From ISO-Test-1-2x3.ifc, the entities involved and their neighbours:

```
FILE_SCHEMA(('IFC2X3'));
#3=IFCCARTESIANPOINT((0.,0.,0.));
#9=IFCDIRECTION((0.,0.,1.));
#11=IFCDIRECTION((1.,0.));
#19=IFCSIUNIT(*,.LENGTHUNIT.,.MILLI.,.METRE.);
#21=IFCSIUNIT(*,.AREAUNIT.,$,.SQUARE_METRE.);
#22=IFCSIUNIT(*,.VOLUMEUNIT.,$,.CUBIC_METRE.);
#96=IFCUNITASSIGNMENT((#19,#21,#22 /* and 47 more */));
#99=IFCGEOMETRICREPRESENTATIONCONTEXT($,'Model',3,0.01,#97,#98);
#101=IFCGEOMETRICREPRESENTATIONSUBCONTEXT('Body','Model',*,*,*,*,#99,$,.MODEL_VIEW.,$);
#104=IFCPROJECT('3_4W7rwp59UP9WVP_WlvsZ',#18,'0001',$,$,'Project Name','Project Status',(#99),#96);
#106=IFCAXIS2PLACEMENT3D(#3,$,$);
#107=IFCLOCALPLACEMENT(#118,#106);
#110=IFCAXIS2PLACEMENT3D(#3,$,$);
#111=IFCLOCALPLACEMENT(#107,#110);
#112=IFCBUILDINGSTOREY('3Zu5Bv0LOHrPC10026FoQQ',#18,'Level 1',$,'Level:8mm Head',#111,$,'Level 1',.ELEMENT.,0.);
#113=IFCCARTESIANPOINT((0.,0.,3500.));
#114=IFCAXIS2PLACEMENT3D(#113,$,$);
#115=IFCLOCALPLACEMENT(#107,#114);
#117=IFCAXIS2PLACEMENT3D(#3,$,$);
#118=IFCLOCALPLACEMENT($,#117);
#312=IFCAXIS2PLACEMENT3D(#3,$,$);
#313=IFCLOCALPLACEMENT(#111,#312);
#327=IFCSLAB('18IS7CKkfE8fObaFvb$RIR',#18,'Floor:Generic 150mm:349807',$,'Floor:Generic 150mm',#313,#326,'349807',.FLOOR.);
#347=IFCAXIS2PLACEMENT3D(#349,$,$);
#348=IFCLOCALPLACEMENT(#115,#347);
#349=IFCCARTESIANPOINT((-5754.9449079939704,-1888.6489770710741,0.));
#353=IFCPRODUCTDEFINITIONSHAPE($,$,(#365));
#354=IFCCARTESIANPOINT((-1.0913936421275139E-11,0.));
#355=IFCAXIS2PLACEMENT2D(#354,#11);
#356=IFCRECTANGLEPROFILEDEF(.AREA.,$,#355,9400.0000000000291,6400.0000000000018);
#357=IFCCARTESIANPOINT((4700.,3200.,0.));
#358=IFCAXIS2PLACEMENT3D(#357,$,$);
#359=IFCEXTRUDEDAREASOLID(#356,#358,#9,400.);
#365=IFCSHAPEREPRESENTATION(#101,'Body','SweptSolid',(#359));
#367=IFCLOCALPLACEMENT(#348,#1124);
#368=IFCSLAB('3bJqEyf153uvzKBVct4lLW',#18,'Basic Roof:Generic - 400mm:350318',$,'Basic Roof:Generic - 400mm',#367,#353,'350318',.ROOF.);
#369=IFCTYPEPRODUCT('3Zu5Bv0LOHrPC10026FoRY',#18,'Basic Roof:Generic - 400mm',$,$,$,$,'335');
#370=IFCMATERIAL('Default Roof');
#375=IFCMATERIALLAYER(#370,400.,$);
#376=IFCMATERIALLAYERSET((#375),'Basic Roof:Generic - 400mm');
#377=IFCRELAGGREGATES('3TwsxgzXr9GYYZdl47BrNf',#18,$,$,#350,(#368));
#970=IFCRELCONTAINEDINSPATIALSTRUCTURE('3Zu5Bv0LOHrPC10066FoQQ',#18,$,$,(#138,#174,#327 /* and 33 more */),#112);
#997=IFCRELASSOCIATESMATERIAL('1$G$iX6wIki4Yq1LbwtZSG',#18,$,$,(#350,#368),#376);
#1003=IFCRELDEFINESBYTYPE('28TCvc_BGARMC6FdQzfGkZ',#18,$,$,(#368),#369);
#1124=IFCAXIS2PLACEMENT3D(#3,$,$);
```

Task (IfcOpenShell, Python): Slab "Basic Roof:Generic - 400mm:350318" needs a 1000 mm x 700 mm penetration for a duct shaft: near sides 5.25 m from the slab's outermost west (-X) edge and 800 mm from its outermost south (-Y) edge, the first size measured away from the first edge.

```python
import numpy as np
import ifcopenshell
import ifcopenshell.api.feature
import ifcopenshell.api.geometry
import ifcopenshell.api.root
import ifcopenshell.geom
import ifcopenshell.util.placement
import ifcopenshell.util.representation
import ifcopenshell.util.shape
import ifcopenshell.util.unit

model = ifcopenshell.open("ISO-Test-1-2x3.ifc")
unit_scale = ifcopenshell.util.unit.calculate_unit_scale(model)
settings = ifcopenshell.geom.settings()


def volume(element):
    """Net volume in cubic metres, openings subtracted."""
    shape = ifcopenshell.geom.create_shape(settings, element)
    return ifcopenshell.util.shape.get_volume(shape.geometry)


slab = model.by_guid("3bJqEyf153uvzKBVct4lLW")
before = volume(slab)

# Extent in the slab's own axes, in metres. The edges named are its -X and -Y sides.
slab_shape = ifcopenshell.geom.create_shape(settings, slab)
vertices = ifcopenshell.util.shape.get_vertices(slab_shape.geometry)
x_min, y_min, bottom = vertices.min(axis=0)
top = vertices[:, 2].max()

opening = ifcopenshell.api.root.create_entity(model, ifc_class="IfcOpeningElement", name="Duct shaft opening")
context = ifcopenshell.util.representation.get_context(model, "Model", "Body", "MODEL_VIEW")
width, depth = 1, 0.7
outline = [(0.0, 0.0), (width, 0.0), (width, depth), (0.0, depth), (0.0, 0.0)]
# Overshoot both faces by 50 mm so the cut is clean.
shape = ifcopenshell.api.geometry.add_slab_representation(
    model, context=context, depth=top - bottom + 0.1, polyline=outline
)
ifcopenshell.api.geometry.assign_representation(model, product=opening, representation=shape)

matrix = ifcopenshell.util.placement.get_local_placement(slab.ObjectPlacement)
matrix[:, 3] = matrix @ np.append(np.array([x_min + 5.25, y_min + 0.8, bottom - 0.05]) / unit_scale, 1.0)
ifcopenshell.api.geometry.edit_object_placement(model, product=opening, matrix=matrix, is_si=False)
ifcopenshell.api.feature.add_feature(model, feature=opening, element=slab)

after = volume(slab)

print(f"slab volume {before:.3f} -> {after:.3f} m3")

model.write("ISO-Test-1-2x3_updated.ifc")
```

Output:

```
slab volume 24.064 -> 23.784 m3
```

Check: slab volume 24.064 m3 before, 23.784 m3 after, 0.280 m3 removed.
